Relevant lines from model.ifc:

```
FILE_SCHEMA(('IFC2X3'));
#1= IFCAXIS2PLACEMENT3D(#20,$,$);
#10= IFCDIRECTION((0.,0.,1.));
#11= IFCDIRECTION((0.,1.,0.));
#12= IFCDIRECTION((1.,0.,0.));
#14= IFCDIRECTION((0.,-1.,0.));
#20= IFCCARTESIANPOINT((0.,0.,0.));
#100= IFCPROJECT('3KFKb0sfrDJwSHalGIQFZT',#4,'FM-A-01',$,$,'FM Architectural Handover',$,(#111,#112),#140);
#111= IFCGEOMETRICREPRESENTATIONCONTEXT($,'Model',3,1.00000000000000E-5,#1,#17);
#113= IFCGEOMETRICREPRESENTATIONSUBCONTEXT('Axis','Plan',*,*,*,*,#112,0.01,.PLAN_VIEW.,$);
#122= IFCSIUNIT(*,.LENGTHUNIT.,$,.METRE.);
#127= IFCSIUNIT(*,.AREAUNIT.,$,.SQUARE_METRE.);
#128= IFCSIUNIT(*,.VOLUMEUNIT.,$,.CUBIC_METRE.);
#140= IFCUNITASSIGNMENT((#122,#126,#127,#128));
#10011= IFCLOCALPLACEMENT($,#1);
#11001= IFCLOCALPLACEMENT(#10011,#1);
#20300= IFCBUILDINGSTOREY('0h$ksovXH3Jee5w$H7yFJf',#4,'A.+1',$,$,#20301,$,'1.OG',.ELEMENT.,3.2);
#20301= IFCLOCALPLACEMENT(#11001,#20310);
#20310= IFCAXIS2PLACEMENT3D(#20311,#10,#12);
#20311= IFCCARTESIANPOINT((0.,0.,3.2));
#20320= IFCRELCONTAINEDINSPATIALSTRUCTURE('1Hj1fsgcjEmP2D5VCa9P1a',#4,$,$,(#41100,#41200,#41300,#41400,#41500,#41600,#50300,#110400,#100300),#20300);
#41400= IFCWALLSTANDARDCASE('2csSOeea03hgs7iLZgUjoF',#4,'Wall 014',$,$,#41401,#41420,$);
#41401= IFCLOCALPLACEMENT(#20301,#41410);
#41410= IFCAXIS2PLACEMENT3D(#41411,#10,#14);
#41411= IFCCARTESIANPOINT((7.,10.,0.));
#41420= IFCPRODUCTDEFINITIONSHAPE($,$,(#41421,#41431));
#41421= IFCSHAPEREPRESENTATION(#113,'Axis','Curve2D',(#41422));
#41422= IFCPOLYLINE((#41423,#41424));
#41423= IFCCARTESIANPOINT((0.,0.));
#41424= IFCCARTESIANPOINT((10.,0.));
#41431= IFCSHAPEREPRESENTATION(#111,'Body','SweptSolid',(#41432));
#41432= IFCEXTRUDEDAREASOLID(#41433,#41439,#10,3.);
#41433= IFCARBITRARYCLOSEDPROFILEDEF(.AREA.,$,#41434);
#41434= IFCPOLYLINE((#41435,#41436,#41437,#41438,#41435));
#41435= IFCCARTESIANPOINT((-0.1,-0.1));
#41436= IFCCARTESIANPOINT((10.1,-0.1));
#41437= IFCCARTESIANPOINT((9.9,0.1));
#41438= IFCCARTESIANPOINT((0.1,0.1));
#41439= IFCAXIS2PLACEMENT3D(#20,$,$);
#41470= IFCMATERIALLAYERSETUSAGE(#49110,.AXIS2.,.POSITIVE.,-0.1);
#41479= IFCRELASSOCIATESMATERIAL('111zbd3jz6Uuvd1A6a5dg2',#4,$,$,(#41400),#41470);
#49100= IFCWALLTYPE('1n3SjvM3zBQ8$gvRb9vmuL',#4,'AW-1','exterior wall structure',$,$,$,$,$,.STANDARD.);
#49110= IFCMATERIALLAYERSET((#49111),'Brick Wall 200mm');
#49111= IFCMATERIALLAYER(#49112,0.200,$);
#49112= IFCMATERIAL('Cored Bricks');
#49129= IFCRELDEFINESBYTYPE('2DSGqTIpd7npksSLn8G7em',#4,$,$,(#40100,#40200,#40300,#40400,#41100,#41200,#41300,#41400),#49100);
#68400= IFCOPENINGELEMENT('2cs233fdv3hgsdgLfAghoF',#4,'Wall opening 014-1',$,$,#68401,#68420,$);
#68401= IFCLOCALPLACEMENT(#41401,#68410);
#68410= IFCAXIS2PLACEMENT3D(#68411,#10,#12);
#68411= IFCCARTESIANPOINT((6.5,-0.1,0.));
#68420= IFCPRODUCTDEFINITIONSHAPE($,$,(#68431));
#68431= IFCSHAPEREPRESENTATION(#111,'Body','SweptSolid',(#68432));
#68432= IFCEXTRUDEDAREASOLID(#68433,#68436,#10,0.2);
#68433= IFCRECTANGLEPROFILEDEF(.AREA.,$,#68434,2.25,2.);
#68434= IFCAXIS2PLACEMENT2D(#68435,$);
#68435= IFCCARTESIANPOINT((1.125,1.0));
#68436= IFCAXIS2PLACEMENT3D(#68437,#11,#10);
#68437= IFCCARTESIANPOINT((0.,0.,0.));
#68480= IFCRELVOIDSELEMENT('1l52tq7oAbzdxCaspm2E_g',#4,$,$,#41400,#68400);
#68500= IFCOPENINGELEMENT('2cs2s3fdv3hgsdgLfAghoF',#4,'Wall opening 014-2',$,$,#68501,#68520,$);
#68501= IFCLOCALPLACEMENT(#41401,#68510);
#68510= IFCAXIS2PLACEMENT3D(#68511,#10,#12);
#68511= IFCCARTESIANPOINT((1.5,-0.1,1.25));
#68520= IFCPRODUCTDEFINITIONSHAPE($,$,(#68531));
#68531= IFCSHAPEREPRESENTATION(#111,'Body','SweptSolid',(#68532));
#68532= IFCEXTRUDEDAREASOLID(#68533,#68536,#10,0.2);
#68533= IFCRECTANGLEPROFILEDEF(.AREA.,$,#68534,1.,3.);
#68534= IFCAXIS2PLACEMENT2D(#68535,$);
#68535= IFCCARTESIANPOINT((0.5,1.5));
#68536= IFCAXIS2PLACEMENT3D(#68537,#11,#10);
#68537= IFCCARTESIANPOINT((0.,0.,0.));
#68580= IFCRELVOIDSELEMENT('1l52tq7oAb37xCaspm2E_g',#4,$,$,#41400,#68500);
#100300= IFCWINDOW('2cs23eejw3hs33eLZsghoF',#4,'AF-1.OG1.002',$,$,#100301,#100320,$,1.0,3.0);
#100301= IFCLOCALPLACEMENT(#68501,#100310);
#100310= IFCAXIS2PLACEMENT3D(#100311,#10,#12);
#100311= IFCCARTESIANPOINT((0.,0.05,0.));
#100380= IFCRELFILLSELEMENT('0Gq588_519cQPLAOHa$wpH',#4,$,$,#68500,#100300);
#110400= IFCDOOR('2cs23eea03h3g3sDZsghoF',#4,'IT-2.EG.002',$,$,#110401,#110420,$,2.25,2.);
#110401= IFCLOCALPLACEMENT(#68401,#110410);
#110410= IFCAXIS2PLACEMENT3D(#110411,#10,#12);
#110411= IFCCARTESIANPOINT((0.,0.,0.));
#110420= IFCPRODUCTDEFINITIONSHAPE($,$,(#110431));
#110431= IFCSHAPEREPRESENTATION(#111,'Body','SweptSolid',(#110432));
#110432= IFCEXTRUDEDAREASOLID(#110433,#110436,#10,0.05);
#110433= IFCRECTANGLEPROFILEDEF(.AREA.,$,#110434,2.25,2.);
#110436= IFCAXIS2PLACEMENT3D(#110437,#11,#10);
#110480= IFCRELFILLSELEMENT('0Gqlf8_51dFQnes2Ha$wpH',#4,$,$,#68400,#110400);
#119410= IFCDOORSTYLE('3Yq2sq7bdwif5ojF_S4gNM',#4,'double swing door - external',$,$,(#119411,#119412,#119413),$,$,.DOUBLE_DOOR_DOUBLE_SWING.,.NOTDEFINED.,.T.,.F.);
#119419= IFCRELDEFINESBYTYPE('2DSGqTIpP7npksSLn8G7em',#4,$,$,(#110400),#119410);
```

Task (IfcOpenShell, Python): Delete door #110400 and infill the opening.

```python
import ifcopenshell
import ifcopenshell.api.feature
import ifcopenshell.api.root
import ifcopenshell.geom
import ifcopenshell.util.shape

model = ifcopenshell.open("model.ifc")
settings = ifcopenshell.geom.settings()


def volume(element):
    """Net volume in cubic metres, openings subtracted."""
    shape = ifcopenshell.geom.create_shape(settings, element)
    return ifcopenshell.util.shape.get_volume(shape.geometry)


door = model.by_guid("2cs23eea03h3g3sDZsghoF")
opening = door.FillsVoids[0].RelatingOpeningElement
wall = opening.VoidsElements[0].RelatingBuildingElement
before = volume(wall)

ifcopenshell.api.root.remove_product(model, product=door)
ifcopenshell.api.feature.remove_feature(model, feature=opening)

after = volume(wall)

print(f"wall volume {before:.3f} -> {after:.3f} m3")

model.write("model_updated.ifc")
```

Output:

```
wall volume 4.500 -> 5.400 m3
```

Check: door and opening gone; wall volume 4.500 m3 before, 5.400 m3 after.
